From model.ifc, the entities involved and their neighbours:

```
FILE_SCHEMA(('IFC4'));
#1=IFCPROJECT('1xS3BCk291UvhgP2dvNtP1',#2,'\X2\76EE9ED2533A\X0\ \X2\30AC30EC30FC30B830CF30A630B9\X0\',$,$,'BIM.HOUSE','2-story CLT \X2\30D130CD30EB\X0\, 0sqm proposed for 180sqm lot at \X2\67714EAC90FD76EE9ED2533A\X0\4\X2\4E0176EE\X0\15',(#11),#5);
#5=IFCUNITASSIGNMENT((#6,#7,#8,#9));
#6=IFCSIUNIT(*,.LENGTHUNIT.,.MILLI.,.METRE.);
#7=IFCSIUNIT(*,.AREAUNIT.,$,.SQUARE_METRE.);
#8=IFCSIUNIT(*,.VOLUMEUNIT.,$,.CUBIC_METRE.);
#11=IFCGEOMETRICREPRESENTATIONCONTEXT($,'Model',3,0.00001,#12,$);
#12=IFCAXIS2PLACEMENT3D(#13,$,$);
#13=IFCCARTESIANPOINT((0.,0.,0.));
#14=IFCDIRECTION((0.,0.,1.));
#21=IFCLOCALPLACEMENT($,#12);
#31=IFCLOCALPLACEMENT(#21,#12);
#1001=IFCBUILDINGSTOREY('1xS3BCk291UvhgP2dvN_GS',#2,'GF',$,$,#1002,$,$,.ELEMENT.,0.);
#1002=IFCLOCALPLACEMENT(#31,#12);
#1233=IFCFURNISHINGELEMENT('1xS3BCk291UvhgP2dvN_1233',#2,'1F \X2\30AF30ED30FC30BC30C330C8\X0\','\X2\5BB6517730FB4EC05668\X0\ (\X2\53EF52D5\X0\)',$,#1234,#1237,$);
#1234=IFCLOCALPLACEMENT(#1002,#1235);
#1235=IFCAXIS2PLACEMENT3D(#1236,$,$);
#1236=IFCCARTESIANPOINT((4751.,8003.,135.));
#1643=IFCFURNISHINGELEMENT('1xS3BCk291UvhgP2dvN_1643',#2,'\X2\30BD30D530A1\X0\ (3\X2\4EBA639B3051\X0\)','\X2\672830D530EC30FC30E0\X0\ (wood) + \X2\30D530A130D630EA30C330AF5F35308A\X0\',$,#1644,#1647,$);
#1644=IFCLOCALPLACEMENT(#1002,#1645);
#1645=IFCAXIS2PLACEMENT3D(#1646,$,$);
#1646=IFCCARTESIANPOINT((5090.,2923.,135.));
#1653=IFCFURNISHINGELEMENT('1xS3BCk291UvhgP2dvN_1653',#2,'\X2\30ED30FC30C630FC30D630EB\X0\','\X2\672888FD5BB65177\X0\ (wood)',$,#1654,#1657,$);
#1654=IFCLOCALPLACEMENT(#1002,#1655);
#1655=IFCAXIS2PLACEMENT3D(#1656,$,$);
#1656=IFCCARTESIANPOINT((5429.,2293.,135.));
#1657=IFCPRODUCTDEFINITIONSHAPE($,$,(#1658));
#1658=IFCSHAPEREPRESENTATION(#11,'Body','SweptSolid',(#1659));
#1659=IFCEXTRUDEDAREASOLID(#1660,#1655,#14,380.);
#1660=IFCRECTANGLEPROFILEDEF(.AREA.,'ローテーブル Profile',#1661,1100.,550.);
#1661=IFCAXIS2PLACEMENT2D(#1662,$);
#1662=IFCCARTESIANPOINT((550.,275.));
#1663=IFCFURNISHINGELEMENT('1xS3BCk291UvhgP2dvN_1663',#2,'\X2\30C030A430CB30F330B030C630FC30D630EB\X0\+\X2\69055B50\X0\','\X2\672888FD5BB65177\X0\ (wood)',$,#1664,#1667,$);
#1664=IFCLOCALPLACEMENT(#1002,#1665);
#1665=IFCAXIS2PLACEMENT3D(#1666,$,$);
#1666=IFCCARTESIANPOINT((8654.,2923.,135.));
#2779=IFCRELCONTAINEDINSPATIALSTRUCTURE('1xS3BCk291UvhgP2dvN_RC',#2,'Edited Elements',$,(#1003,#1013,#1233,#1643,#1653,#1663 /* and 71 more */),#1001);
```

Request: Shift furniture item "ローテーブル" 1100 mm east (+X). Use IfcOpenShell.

```python
import ifcopenshell
import ifcopenshell.api.geometry
import ifcopenshell.util.placement
import ifcopenshell.util.unit

model = ifcopenshell.open("model.ifc")
unit_scale = ifcopenshell.util.unit.calculate_unit_scale(model)

item = model.by_guid("1xS3BCk291UvhgP2dvN_1653")
matrix = ifcopenshell.util.placement.get_local_placement(item.ObjectPlacement)
matrix[0, 3] += 1.1 / unit_scale
ifcopenshell.api.geometry.edit_object_placement(model, product=item, matrix=matrix, is_si=False)

print(ifcopenshell.util.placement.get_local_placement(item.ObjectPlacement).round(3) + 0.0)

model.write("model_updated.ifc")
```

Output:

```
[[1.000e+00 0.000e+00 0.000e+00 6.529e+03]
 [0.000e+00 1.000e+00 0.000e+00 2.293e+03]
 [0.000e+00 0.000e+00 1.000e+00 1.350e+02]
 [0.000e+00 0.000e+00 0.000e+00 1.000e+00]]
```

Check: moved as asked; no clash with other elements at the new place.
